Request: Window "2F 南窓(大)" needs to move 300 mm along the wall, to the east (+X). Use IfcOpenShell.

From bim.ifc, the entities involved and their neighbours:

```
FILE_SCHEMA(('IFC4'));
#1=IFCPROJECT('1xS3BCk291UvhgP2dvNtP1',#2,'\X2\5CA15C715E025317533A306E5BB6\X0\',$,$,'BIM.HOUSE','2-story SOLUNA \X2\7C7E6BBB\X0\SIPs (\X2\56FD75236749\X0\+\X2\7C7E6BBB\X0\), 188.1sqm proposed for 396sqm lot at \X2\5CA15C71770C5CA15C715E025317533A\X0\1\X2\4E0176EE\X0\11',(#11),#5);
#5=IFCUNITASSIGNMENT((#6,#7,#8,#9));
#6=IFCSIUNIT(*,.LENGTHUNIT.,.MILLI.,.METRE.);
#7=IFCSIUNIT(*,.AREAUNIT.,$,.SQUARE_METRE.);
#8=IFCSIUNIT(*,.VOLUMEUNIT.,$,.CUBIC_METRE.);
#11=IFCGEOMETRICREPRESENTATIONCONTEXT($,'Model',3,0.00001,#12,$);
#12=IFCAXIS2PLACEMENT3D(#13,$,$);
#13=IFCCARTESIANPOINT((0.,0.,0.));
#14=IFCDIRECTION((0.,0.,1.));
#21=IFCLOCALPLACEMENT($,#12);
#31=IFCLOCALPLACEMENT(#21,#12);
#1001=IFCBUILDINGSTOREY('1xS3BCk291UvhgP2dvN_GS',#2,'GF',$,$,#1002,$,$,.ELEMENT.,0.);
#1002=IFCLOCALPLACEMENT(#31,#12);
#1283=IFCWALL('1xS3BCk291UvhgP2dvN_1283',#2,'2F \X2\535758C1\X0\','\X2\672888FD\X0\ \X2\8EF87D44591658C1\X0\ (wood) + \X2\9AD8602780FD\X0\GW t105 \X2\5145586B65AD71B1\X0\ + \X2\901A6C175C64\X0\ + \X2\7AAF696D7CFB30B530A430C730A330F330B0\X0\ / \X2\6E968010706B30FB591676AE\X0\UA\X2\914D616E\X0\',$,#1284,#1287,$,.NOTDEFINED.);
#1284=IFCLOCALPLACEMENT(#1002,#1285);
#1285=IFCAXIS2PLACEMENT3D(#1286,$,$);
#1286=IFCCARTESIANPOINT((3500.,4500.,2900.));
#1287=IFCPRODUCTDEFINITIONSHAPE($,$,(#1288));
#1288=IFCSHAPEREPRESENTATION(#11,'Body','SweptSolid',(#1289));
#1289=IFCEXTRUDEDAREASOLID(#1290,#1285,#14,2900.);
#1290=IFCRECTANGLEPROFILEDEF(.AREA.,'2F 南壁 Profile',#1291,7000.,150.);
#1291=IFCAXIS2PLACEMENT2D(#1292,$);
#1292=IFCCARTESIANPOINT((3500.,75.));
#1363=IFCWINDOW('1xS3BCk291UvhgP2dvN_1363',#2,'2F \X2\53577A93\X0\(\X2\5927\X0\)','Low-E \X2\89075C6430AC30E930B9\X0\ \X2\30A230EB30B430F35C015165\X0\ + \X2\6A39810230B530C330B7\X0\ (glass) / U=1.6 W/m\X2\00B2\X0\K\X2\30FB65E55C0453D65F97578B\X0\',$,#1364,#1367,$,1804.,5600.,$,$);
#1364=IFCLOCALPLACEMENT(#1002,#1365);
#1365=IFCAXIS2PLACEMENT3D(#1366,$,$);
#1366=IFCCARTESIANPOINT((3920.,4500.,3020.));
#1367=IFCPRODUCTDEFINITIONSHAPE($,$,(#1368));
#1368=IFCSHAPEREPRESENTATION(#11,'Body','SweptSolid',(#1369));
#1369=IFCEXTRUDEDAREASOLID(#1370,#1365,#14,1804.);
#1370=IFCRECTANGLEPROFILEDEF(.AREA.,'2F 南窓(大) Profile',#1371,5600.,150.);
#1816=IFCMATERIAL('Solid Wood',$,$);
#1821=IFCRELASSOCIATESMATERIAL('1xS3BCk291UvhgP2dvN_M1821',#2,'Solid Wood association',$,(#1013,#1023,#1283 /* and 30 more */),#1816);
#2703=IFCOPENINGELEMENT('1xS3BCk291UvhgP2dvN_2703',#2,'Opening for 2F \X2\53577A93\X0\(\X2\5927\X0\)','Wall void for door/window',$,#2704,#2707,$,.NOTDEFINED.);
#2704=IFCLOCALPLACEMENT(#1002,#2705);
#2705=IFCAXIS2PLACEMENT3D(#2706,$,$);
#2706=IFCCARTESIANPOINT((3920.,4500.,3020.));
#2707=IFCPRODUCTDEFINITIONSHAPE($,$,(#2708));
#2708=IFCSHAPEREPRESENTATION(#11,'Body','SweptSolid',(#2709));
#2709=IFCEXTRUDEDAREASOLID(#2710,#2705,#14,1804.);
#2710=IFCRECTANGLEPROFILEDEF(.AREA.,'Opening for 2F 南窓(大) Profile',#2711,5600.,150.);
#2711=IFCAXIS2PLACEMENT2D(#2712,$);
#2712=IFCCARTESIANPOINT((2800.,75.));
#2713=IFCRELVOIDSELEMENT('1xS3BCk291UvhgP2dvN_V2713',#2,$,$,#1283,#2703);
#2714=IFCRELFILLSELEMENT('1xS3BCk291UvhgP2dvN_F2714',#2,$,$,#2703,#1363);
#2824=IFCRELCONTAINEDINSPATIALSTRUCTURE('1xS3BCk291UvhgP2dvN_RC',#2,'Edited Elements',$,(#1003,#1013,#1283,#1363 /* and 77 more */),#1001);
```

```python
import ifcopenshell
import ifcopenshell.api.geometry
import ifcopenshell.util.placement

model = ifcopenshell.open("bim.ifc")

window = model.by_guid("1xS3BCk291UvhgP2dvN_1363")
opening = window.FillsVoids[0].RelatingOpeningElement
wall = opening.VoidsElements[0].RelatingBuildingElement

wall_matrix = ifcopenshell.util.placement.get_local_placement(wall.ObjectPlacement)
shift = wall_matrix[:3, 0] * 300.0
before = ifcopenshell.util.placement.get_local_placement(window.ObjectPlacement)[:3, 3].copy()

# The window is not placed relative to its opening, so move both.
for product in (opening, window):
    matrix = ifcopenshell.util.placement.get_local_placement(product.ObjectPlacement)
    matrix[:3, 3] += shift
    ifcopenshell.api.geometry.edit_object_placement(model, product=product, matrix=matrix, is_si=False)

after = ifcopenshell.util.placement.get_local_placement(window.ObjectPlacement)[:3, 3]
print("window moved by", (after - before).round(3) + 0.0)

model.write("bim-out.ifc")
```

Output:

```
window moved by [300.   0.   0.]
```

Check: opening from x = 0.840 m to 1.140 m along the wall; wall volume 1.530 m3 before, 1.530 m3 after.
